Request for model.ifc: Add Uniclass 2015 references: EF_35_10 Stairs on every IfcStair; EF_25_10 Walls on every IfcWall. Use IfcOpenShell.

First a look at what the model holds.

```python
import ifcopenshell

model = ifcopenshell.open("model.ifc")
print(model.schema)
print("classifications:", [c.Name for c in model.by_type("IfcClassification")])
for ifc_class in ("IfcDoor", "IfcRoof", "IfcStair", "IfcWall", "IfcWindow"):
    print(ifc_class, len(model.by_type(ifc_class)))
```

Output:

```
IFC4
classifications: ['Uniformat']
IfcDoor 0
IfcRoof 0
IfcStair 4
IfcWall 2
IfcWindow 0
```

```python
import ifcopenshell
import ifcopenshell.api.classification

model = ifcopenshell.open("model.ifc")

system = ifcopenshell.api.classification.add_classification(model, classification="Uniclass 2015")

codes = {
    "IfcStair": ("EF_35_10", "Stairs"),
    "IfcWall": ("EF_25_10", "Walls"),
}
for ifc_class, (code, name) in codes.items():
    products = model.by_type(ifc_class)
    ifcopenshell.api.classification.add_reference(
        model, products=products, classification=system, identification=code, name=name
    )
    print(code, len(products))

model.write("model_v2.ifc")
```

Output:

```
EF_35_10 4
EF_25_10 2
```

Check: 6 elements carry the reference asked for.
